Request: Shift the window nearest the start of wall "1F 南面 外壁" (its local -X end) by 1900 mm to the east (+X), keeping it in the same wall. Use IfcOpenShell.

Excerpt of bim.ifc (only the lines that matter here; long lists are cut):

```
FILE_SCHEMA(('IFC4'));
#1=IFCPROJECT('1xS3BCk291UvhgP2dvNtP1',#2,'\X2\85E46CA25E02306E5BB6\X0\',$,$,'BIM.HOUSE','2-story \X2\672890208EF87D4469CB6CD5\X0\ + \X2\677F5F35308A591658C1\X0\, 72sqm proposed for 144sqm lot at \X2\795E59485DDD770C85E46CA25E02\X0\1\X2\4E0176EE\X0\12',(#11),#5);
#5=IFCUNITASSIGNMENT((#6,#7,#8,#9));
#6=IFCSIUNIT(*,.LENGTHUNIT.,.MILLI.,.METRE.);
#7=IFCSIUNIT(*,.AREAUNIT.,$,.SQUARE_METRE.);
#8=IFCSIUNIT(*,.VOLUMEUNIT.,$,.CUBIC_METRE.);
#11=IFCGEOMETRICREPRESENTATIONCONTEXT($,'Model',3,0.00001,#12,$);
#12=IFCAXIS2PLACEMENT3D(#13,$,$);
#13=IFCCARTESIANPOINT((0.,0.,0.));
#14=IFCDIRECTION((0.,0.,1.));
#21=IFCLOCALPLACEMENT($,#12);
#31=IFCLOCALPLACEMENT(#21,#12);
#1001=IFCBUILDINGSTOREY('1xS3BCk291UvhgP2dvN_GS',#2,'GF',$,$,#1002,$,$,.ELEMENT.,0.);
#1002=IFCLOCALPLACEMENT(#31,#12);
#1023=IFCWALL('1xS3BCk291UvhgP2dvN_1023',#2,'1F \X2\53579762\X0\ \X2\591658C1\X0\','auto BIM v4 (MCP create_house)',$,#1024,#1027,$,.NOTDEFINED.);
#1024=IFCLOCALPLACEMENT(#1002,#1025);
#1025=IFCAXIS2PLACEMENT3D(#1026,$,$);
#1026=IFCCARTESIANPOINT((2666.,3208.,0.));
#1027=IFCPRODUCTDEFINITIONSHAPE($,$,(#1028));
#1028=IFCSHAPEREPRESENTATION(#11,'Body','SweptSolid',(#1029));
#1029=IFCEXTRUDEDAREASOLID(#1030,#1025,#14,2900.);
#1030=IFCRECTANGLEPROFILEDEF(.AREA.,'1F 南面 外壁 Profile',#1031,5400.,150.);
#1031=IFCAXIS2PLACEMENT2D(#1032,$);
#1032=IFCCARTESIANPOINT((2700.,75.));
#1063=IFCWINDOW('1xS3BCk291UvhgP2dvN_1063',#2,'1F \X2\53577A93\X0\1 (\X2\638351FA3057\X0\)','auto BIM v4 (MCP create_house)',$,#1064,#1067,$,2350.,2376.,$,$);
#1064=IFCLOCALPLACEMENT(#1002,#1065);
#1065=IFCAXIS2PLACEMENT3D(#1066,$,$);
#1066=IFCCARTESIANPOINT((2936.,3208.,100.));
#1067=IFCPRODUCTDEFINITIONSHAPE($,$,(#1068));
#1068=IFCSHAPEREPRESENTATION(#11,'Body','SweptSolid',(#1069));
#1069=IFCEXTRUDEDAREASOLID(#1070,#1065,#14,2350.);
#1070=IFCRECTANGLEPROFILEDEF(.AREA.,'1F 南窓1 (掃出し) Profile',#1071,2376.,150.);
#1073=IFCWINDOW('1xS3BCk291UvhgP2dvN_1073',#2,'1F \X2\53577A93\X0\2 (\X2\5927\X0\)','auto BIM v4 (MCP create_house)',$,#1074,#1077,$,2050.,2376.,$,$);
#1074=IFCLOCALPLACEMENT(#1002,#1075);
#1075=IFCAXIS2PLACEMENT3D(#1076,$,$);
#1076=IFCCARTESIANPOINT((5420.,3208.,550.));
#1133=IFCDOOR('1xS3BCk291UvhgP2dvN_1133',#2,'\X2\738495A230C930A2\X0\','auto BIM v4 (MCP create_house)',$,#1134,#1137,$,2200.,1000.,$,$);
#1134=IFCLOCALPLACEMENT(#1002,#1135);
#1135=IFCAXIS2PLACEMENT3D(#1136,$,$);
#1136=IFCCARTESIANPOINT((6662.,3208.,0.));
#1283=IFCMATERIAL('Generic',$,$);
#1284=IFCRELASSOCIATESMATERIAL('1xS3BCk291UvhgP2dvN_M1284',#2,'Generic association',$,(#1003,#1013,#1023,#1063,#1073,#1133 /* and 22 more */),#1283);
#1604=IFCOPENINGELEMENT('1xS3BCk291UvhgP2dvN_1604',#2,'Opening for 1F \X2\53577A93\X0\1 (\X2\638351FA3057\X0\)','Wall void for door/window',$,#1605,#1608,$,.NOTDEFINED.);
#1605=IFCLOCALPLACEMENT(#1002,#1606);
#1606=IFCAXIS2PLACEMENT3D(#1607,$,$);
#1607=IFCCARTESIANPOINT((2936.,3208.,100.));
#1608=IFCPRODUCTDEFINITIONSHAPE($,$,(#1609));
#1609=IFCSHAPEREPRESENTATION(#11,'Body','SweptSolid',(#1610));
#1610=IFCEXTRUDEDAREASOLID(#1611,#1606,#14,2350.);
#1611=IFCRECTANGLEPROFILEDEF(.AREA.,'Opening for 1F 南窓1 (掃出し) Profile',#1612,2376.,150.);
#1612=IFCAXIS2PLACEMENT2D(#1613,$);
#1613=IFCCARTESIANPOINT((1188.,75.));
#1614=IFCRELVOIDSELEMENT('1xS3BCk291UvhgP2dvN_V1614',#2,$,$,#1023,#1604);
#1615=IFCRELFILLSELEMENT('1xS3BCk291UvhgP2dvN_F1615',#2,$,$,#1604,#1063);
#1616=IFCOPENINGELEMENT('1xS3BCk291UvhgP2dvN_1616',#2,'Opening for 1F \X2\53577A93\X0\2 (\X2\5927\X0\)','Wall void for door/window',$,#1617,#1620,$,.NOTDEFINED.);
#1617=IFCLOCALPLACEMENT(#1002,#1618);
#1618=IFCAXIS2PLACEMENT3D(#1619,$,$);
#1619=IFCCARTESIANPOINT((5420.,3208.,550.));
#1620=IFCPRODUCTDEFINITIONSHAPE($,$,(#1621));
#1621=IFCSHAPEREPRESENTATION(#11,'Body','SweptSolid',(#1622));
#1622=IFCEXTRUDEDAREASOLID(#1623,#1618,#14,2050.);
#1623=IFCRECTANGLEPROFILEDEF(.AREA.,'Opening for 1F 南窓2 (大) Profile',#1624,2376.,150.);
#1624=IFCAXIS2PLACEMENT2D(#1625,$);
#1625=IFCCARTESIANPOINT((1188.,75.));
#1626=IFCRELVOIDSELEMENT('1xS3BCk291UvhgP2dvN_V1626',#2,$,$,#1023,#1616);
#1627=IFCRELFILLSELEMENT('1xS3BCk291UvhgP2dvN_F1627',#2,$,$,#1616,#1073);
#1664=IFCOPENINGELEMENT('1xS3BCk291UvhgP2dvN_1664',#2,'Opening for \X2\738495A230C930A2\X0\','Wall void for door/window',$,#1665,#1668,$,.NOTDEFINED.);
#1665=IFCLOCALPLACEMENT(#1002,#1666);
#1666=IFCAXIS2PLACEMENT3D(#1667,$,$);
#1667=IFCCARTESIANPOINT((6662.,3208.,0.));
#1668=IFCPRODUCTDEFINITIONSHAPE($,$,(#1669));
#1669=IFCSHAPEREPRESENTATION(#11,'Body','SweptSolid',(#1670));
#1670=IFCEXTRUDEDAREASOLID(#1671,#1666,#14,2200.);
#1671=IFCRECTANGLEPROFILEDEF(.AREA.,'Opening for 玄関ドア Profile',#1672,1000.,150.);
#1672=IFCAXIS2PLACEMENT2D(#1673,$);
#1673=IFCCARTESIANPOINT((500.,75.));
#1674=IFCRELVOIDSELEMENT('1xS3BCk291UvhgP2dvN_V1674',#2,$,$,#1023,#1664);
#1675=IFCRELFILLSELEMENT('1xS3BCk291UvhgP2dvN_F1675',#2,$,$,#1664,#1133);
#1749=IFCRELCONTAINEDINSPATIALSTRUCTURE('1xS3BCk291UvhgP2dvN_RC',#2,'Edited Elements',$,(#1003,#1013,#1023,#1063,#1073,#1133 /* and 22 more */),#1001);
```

```python
import ifcopenshell
import ifcopenshell.api.geometry
import ifcopenshell.util.placement
import ifcopenshell.util.unit

model = ifcopenshell.open("bim.ifc")
unit_scale = ifcopenshell.util.unit.calculate_unit_scale(model)

window = model.by_guid("1xS3BCk291UvhgP2dvN_1063")
opening = window.FillsVoids[0].RelatingOpeningElement
wall = opening.VoidsElements[0].RelatingBuildingElement

wall_matrix = ifcopenshell.util.placement.get_local_placement(wall.ObjectPlacement)
shift = wall_matrix[:3, 0] * 1.9 / unit_scale
before = ifcopenshell.util.placement.get_local_placement(window.ObjectPlacement)[:3, 3].copy()

# The window is not placed relative to its opening, so move both.
for product in (opening, window):
    matrix = ifcopenshell.util.placement.get_local_placement(product.ObjectPlacement)
    matrix[:3, 3] += shift
    ifcopenshell.api.geometry.edit_object_placement(model, product=product, matrix=matrix, is_si=False)

after = ifcopenshell.util.placement.get_local_placement(window.ObjectPlacement)[:3, 3]
print("window moved by", (after - before).round(3) + 0.0)

model.write("bim-out.ifc")
```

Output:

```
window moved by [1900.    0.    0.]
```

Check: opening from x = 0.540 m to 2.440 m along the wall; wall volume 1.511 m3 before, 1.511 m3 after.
